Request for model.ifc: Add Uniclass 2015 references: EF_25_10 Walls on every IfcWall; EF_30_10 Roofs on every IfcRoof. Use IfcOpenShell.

First a look at what the model holds.

```python
import ifcopenshell

model = ifcopenshell.open("model.ifc")
print(model.schema)
print("classifications:", [c.Name for c in model.by_type("IfcClassification")])
for ifc_class in ("IfcDoor", "IfcRoof", "IfcStair", "IfcWall", "IfcWindow"):
    print(ifc_class, len(model.by_type(ifc_class)))
```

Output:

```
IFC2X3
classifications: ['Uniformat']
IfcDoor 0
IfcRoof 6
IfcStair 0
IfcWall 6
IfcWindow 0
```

```python
import ifcopenshell
import ifcopenshell.api.classification

model = ifcopenshell.open("model.ifc")

# IFC2X3 requires Source and Edition and has no link from the project to the system.
system = model.create_entity("IfcClassification", Source="NBS", Edition="2015", Name="Uniclass 2015")

codes = {
    "IfcWall": ("EF_25_10", "Walls"),
    "IfcRoof": ("EF_30_10", "Roofs"),
}
for ifc_class, (code, name) in codes.items():
    products = model.by_type(ifc_class)
    ifcopenshell.api.classification.add_reference(
        model, products=products, classification=system, identification=code, name=name
    )
    print(code, len(products))

model.write("model_updated.ifc")
```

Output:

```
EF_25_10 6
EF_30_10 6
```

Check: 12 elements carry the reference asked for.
